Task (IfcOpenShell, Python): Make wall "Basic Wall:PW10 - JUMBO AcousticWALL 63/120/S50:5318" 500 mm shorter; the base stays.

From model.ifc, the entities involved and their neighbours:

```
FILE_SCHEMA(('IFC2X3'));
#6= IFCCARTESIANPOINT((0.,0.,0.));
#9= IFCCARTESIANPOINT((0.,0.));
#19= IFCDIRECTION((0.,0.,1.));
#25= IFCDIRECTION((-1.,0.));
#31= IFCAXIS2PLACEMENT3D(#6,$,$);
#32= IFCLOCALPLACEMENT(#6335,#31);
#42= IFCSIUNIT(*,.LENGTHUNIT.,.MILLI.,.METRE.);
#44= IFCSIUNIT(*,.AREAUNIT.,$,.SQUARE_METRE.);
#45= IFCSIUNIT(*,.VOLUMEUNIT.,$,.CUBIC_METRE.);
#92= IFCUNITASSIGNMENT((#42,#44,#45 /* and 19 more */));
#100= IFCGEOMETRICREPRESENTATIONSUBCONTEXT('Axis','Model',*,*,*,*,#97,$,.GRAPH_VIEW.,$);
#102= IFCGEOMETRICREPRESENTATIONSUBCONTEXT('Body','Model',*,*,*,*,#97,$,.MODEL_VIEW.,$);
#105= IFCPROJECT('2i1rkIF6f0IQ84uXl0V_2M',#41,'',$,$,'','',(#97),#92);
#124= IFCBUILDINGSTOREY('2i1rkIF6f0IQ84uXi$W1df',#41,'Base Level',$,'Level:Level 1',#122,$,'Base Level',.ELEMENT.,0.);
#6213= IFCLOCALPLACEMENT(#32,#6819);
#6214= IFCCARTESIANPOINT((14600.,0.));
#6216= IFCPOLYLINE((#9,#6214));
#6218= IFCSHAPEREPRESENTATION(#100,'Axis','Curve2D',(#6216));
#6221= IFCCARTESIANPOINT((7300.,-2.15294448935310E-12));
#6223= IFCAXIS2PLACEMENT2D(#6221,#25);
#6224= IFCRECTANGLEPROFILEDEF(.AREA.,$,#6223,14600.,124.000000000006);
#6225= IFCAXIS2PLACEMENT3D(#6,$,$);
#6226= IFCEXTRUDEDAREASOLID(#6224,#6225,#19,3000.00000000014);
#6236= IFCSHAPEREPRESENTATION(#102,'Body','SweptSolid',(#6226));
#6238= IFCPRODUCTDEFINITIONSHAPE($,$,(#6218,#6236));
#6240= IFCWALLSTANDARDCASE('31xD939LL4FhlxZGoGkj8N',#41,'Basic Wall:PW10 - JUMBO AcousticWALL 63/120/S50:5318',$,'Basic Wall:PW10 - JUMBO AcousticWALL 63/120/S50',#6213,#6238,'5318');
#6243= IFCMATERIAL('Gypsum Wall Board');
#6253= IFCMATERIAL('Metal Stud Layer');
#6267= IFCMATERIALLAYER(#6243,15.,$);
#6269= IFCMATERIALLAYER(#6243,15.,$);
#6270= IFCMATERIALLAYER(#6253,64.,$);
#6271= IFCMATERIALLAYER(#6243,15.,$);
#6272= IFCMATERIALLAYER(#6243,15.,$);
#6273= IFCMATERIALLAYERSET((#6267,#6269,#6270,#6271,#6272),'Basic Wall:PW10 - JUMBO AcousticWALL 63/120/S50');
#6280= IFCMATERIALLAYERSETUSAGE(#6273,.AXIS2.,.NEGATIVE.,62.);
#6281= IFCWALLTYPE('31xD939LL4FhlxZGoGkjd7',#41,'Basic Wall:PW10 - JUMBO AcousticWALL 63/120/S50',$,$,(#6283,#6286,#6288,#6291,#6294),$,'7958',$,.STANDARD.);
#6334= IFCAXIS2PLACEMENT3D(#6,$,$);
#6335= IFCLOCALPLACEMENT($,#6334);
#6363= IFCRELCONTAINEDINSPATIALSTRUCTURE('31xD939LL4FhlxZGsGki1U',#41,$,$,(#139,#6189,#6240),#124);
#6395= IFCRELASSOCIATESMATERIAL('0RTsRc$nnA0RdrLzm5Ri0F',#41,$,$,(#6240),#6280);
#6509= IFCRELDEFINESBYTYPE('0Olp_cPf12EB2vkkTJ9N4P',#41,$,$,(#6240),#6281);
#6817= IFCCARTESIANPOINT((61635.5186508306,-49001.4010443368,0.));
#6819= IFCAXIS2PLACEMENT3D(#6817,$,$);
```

```python
import ifcopenshell
import ifcopenshell.geom
import ifcopenshell.util.representation
import ifcopenshell.util.shape
import ifcopenshell.util.unit

model = ifcopenshell.open("model.ifc")
unit_scale = ifcopenshell.util.unit.calculate_unit_scale(model)
settings = ifcopenshell.geom.settings()


def volume(element):
    """Net volume in cubic metres, openings subtracted."""
    shape = ifcopenshell.geom.create_shape(settings, element)
    return ifcopenshell.util.shape.get_volume(shape.geometry)


wall = model.by_guid("31xD939LL4FhlxZGoGkj8N")
before = volume(wall)

body = ifcopenshell.util.representation.get_representation(wall, "Model", "Body")
solid = body.Items[0]
old_height = solid.Depth
solid.Depth -= 0.5 / unit_scale
after = volume(wall)

print(f"height {old_height:g} -> {solid.Depth:g}, volume {before:.3f} -> {after:.3f} m3")

model.write("model_v2.ifc")
```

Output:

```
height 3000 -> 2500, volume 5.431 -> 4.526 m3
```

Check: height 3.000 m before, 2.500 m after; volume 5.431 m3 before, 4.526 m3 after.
